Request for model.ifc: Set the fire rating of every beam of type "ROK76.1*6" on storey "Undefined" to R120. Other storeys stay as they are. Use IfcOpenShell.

First a look at what the model holds.

```python
import ifcopenshell
import ifcopenshell.util.element

model = ifcopenshell.open("model.ifc")
print(model.schema)
storey = next(s for s in model.by_type("IfcBuildingStorey") if s.Name == "Undefined")
beams = [e for e in ifcopenshell.util.element.get_decomposition(storey) if e.is_a("IfcBeam")]
seen = {}
for e in beams:
    element_type = ifcopenshell.util.element.get_type(e)
    key = (element_type.Name if element_type != e and element_type else None, ifcopenshell.util.element.get_pset(e, "Pset_BeamCommon", "FireRating"))
    seen[key] = seen.get(key, 0) + 1
for (name, value), count in sorted(seen.items(), key=str):
    print(count, "x", name, "|", value)
```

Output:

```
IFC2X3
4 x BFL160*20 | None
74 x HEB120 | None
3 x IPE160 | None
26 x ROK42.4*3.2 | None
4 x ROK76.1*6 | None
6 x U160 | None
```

```python
import ifcopenshell
import ifcopenshell.api.pset
import ifcopenshell.util.element

model = ifcopenshell.open("model.ifc")

storey = next(s for s in model.by_type("IfcBuildingStorey") if s.Name == "Undefined")
beams = [e for e in ifcopenshell.util.element.get_decomposition(storey) if e.is_a("IfcBeam")]

count = 0
for e in beams:
    element_type = ifcopenshell.util.element.get_type(e)
    if element_type in (None, e) or element_type.Name != "ROK76.1*6":
        continue
    # add_pset returns the element's existing set when there is one.
    pset = ifcopenshell.api.pset.add_pset(model, product=e, name="Pset_BeamCommon")
    ifcopenshell.api.pset.edit_pset(model, pset=pset, properties={"FireRating": "R120"})
    count += 1

print(count, "beams updated")

model.write("model_rev.ifc")
```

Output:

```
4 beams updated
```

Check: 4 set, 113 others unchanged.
